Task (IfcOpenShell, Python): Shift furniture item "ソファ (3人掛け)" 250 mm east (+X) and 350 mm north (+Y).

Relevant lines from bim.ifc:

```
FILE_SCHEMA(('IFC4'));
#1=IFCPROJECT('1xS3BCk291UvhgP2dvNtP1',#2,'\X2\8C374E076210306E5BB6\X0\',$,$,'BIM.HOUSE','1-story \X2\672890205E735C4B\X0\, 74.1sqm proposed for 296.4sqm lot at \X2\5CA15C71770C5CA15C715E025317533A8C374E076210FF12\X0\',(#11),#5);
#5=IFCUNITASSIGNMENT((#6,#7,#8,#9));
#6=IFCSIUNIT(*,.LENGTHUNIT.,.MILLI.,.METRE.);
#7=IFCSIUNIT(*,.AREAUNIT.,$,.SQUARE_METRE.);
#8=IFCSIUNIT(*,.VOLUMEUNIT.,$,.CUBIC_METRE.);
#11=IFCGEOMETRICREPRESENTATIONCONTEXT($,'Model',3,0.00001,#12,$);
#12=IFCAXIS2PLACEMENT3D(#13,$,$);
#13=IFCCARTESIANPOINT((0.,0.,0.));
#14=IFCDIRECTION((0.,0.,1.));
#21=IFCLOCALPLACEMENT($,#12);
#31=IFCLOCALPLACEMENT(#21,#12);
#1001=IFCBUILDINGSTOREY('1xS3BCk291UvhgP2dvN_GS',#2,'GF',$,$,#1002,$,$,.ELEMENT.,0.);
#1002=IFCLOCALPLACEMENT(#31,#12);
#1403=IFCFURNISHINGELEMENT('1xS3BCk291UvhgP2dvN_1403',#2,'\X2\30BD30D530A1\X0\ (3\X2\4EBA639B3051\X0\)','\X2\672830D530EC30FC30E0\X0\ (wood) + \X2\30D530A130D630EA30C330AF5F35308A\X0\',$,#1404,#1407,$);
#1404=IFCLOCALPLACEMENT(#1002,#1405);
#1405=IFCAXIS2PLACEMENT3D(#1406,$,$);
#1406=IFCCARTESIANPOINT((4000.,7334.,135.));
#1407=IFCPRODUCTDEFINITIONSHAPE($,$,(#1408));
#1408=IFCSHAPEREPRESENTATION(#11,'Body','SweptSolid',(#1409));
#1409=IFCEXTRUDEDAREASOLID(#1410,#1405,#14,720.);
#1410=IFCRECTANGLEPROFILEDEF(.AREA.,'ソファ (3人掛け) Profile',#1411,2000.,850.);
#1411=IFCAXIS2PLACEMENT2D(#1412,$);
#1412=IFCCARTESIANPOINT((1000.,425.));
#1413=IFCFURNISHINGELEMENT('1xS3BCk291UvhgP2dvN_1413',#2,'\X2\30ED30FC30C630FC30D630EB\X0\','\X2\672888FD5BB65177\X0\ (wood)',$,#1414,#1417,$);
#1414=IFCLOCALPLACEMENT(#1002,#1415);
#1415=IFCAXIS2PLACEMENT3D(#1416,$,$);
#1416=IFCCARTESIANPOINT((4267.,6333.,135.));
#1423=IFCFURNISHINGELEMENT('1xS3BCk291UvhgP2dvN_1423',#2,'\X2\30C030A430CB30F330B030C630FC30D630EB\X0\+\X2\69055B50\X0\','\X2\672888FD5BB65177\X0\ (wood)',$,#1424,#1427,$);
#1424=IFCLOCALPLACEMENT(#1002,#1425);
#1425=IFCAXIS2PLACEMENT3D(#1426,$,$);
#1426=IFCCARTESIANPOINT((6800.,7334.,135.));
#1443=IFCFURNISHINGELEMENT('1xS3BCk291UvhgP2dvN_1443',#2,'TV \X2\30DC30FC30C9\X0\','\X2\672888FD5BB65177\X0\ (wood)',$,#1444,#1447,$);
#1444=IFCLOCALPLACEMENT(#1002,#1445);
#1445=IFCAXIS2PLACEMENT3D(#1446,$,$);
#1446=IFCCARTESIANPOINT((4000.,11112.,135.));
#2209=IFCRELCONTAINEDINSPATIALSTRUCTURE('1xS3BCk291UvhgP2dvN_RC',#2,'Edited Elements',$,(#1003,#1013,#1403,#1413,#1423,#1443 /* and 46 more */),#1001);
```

```python
import ifcopenshell
import ifcopenshell.api.geometry
import ifcopenshell.util.placement
import ifcopenshell.util.unit

model = ifcopenshell.open("bim.ifc")
unit_scale = ifcopenshell.util.unit.calculate_unit_scale(model)

item = model.by_guid("1xS3BCk291UvhgP2dvN_1403")
matrix = ifcopenshell.util.placement.get_local_placement(item.ObjectPlacement)
matrix[0, 3] += 0.25 / unit_scale
matrix[1, 3] += 0.35 / unit_scale
ifcopenshell.api.geometry.edit_object_placement(model, product=item, matrix=matrix, is_si=False)

print(ifcopenshell.util.placement.get_local_placement(item.ObjectPlacement).round(3) + 0.0)

model.write("bim_edited.ifc")
```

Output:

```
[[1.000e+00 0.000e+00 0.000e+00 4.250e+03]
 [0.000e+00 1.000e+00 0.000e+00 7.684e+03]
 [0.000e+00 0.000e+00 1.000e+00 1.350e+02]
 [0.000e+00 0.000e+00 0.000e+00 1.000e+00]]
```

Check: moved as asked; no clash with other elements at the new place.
